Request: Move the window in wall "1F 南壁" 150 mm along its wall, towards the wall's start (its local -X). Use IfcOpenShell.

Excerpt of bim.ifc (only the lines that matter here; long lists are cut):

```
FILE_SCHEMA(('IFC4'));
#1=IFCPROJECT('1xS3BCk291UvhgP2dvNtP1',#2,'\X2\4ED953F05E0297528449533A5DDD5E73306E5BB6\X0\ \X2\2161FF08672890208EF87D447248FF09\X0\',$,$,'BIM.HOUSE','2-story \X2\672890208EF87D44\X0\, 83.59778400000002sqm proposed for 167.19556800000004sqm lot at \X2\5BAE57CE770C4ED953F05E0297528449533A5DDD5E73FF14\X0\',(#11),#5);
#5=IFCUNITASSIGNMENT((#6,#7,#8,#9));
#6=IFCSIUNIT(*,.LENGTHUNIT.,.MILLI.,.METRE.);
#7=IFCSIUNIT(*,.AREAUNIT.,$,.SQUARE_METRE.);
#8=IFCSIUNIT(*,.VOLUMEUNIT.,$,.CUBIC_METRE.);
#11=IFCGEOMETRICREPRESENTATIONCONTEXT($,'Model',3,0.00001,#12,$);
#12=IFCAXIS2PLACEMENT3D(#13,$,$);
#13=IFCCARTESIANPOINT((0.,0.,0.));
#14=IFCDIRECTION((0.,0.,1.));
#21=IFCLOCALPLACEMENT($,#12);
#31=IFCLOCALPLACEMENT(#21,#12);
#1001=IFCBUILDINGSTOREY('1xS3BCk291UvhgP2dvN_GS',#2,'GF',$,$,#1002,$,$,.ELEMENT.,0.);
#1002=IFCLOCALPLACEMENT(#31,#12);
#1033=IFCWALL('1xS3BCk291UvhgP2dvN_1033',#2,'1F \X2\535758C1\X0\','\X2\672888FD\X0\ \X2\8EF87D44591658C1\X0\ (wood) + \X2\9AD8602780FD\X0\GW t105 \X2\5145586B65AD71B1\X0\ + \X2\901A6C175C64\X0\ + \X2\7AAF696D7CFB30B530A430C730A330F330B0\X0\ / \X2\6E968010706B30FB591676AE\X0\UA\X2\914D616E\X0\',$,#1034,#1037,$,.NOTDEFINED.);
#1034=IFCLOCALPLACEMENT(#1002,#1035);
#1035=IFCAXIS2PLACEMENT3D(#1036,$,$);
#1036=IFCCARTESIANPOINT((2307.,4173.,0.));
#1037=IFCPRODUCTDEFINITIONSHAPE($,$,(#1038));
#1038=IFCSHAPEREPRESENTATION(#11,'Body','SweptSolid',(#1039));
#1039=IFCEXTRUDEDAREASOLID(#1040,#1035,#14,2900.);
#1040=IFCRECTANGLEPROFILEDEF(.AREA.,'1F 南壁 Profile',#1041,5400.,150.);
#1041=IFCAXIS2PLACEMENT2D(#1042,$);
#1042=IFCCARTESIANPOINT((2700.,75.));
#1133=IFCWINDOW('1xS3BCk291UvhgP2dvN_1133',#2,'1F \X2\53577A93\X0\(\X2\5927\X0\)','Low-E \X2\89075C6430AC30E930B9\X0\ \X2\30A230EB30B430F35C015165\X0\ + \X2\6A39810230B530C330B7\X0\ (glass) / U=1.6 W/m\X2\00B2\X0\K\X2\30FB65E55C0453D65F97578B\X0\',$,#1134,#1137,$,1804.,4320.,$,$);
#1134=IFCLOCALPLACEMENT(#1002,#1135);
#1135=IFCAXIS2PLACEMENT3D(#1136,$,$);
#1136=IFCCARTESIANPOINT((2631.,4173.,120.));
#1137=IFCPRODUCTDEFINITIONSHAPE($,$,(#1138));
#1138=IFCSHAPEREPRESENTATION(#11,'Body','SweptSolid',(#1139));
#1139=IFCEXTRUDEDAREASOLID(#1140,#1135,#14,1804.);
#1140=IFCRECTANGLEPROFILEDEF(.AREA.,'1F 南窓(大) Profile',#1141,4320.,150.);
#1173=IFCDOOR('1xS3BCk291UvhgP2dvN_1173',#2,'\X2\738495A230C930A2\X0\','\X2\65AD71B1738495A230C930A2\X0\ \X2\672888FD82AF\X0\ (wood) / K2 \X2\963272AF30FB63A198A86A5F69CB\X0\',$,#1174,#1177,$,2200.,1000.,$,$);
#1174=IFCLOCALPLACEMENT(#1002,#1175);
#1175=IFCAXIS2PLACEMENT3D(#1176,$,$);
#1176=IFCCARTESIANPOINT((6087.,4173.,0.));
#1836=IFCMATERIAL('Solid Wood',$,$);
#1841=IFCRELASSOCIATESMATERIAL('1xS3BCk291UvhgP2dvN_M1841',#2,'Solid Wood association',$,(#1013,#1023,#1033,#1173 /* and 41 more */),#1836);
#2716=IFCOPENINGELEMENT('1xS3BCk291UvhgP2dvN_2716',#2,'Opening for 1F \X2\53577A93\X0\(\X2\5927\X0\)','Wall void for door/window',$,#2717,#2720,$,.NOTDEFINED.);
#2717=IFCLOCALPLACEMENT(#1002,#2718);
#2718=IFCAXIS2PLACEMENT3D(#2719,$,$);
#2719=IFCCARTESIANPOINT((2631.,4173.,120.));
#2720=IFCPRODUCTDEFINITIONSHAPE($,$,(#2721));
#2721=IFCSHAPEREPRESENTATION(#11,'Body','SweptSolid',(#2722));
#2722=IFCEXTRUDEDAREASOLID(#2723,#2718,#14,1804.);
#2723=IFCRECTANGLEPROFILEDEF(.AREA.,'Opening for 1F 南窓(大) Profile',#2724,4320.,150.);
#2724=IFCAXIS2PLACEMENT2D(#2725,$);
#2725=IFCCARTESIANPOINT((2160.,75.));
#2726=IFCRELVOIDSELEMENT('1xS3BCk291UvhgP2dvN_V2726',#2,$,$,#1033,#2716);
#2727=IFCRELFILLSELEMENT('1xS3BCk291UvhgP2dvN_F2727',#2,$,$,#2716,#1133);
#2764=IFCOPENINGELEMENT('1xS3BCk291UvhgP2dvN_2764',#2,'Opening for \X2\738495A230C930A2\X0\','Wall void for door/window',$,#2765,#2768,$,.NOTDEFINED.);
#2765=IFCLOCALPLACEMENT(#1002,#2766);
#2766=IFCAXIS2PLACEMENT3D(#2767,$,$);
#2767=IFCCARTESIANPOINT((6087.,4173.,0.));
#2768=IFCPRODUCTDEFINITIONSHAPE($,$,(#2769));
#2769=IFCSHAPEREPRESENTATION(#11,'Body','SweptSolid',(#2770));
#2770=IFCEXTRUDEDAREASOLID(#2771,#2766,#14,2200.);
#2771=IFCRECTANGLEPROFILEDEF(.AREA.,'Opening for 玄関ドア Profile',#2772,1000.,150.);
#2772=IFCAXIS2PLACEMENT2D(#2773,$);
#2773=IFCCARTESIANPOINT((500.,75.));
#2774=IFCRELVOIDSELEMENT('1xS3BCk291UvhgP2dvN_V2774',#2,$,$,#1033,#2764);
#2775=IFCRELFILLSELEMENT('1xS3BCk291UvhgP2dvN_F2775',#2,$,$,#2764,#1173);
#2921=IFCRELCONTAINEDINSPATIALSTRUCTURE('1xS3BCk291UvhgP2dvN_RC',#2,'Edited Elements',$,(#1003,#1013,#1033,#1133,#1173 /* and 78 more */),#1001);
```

```python
import ifcopenshell
import ifcopenshell.api.geometry
import ifcopenshell.util.placement

model = ifcopenshell.open("bim.ifc")

window = model.by_id(1133)
opening = window.FillsVoids[0].RelatingOpeningElement
wall = opening.VoidsElements[0].RelatingBuildingElement

wall_matrix = ifcopenshell.util.placement.get_local_placement(wall.ObjectPlacement)
shift = wall_matrix[:3, 0] * -150.0
before = ifcopenshell.util.placement.get_local_placement(window.ObjectPlacement)[:3, 3].copy()

# The window is not placed relative to its opening, so move both.
for product in (opening, window):
    matrix = ifcopenshell.util.placement.get_local_placement(product.ObjectPlacement)
    matrix[:3, 3] += shift
    ifcopenshell.api.geometry.edit_object_placement(model, product=product, matrix=matrix, is_si=False)

after = ifcopenshell.util.placement.get_local_placement(window.ObjectPlacement)[:3, 3]
print("window moved by", (after - before).round(3) + 0.0)

model.write("bim_rev.ifc")
```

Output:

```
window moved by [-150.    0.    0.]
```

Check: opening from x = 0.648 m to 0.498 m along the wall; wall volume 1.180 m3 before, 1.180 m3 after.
